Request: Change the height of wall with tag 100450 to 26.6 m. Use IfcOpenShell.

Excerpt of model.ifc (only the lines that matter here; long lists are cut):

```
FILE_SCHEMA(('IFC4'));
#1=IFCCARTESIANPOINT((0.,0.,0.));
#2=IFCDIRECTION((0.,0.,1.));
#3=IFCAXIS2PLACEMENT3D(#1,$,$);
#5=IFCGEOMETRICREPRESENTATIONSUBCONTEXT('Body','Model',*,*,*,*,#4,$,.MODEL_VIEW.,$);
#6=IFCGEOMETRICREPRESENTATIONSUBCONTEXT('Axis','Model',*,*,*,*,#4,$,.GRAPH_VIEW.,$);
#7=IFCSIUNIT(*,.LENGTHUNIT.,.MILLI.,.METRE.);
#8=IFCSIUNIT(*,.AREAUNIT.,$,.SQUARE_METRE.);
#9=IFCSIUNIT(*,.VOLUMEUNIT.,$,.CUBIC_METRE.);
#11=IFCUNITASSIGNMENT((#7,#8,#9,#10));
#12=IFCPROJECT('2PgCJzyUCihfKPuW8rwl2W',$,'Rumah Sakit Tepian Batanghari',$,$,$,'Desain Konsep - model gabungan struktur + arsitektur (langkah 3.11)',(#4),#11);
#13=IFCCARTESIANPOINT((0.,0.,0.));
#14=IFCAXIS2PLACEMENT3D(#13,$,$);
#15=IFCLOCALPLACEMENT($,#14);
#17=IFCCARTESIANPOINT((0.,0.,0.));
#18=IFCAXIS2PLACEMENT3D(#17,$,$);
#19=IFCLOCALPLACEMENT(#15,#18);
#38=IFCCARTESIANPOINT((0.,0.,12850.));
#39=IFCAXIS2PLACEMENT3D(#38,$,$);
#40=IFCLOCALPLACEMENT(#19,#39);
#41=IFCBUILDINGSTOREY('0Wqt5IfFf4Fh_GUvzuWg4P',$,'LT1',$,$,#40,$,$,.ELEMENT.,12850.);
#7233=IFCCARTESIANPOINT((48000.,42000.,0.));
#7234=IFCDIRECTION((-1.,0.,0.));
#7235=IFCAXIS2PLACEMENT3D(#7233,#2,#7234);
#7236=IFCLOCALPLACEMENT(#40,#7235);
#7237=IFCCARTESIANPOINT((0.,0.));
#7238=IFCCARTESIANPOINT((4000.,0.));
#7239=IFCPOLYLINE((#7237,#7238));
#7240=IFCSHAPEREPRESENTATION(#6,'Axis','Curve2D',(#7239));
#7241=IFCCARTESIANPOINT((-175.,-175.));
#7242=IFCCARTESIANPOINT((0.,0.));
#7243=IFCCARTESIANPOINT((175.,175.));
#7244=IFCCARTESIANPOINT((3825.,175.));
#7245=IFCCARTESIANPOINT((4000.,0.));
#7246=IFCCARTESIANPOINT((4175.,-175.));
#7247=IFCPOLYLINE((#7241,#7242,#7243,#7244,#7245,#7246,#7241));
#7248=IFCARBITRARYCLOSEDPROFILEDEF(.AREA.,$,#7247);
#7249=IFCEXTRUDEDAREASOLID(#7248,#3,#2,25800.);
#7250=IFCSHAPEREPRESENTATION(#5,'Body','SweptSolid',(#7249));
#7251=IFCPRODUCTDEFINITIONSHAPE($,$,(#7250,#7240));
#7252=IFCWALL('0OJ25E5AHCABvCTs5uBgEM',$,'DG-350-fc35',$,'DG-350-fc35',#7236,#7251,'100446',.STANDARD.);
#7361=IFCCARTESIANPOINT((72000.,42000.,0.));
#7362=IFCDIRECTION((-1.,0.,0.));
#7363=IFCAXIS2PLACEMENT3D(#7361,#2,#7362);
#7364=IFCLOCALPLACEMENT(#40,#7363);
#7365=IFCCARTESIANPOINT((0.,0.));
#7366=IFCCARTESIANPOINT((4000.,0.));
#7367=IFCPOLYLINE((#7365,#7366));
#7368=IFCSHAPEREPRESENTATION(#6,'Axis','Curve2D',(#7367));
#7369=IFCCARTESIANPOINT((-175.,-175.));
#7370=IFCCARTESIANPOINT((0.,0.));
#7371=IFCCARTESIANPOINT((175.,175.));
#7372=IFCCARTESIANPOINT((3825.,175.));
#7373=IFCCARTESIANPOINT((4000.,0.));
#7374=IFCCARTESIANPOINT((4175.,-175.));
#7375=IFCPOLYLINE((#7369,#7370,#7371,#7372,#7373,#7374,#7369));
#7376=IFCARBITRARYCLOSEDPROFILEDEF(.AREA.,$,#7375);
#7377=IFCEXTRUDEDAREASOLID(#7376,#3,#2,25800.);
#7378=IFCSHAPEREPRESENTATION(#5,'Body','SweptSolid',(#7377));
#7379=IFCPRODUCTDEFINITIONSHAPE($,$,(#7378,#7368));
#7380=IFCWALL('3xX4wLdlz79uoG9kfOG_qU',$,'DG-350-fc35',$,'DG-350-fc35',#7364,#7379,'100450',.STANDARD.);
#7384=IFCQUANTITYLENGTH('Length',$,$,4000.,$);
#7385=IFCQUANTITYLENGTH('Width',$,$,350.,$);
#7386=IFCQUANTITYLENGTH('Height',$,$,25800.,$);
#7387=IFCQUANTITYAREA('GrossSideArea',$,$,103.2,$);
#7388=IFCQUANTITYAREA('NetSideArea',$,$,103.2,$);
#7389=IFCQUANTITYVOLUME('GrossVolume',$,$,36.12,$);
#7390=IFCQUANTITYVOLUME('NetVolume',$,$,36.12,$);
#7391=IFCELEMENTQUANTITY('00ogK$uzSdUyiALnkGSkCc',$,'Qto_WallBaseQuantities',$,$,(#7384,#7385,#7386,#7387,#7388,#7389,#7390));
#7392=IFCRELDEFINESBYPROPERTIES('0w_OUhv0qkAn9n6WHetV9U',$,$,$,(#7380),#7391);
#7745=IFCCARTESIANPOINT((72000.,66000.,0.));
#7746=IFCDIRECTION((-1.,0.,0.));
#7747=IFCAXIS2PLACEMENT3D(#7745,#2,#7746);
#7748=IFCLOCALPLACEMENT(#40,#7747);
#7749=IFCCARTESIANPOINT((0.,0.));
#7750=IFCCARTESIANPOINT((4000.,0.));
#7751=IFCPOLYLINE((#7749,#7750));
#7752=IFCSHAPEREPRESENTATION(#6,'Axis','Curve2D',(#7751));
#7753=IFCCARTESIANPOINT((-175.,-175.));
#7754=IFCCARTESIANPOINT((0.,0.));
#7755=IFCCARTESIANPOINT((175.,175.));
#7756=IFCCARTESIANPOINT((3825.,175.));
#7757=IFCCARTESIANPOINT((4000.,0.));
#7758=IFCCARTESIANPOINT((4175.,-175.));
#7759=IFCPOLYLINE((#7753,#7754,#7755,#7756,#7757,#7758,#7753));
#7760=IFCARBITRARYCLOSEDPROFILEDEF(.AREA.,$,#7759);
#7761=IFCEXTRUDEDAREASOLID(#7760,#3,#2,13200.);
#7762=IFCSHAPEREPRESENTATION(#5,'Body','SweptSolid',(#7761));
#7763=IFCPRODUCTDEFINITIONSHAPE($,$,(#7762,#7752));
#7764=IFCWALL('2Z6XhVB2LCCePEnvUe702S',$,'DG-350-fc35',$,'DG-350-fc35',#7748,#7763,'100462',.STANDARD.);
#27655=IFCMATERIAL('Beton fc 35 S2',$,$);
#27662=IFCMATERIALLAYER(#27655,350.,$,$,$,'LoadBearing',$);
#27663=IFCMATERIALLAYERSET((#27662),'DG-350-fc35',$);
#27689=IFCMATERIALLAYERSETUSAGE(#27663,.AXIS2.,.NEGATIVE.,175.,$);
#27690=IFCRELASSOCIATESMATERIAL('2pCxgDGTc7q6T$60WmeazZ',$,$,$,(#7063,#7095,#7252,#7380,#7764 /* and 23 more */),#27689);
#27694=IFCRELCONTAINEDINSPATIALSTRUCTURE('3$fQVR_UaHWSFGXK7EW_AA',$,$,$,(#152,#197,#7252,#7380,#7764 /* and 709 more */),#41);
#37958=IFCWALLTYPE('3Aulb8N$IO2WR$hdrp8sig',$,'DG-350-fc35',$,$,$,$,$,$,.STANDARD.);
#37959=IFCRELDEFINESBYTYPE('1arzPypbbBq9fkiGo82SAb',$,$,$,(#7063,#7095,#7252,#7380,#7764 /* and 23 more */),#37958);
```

```python
import ifcopenshell
import ifcopenshell.api.pset
import ifcopenshell.geom
import ifcopenshell.util.element
import ifcopenshell.util.representation
import ifcopenshell.util.shape
import ifcopenshell.util.unit

model = ifcopenshell.open("model.ifc")
unit_scale = ifcopenshell.util.unit.calculate_unit_scale(model)
area_scale = ifcopenshell.util.unit.calculate_unit_scale(model, "AREAUNIT")
volume_scale = ifcopenshell.util.unit.calculate_unit_scale(model, "VOLUMEUNIT")
settings = ifcopenshell.geom.settings()


def volume(element):
    """Net volume in cubic metres, openings subtracted."""
    shape = ifcopenshell.geom.create_shape(settings, element)
    return ifcopenshell.util.shape.get_volume(shape.geometry)


wall = model.by_guid("3xX4wLdlz79uoG9kfOG_qU")
before = volume(wall)

body = ifcopenshell.util.representation.get_representation(wall, "Model", "Body")
solid = body.Items[0]
old_height = solid.Depth
solid.Depth = 26.6 / unit_scale
after = volume(wall)
thickness = 0.35  # wall thickness in metres

# Update the stored height, areas and volumes.
qto = model.by_id(ifcopenshell.util.element.get_pset(wall, "Qto_WallBaseQuantities", should_inherit=False)["id"])
ifcopenshell.api.pset.edit_qto(model, qto=qto, properties={
    "Height": solid.Depth,
    "GrossSideArea": ifcopenshell.util.element.get_pset(wall, "Qto_WallBaseQuantities", "GrossSideArea") * solid.Depth / old_height,
    "NetSideArea": after / thickness / area_scale,
    "GrossVolume": ifcopenshell.util.element.get_pset(wall, "Qto_WallBaseQuantities", "GrossVolume") * solid.Depth / old_height,
    "NetVolume": after / volume_scale,
})

print(f"height {old_height:g} -> {solid.Depth:g}, volume {before:.3f} -> {after:.3f} m3")

model.write("model_edited.ifc")
```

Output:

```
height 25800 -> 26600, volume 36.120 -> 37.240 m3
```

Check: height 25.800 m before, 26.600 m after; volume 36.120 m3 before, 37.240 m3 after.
